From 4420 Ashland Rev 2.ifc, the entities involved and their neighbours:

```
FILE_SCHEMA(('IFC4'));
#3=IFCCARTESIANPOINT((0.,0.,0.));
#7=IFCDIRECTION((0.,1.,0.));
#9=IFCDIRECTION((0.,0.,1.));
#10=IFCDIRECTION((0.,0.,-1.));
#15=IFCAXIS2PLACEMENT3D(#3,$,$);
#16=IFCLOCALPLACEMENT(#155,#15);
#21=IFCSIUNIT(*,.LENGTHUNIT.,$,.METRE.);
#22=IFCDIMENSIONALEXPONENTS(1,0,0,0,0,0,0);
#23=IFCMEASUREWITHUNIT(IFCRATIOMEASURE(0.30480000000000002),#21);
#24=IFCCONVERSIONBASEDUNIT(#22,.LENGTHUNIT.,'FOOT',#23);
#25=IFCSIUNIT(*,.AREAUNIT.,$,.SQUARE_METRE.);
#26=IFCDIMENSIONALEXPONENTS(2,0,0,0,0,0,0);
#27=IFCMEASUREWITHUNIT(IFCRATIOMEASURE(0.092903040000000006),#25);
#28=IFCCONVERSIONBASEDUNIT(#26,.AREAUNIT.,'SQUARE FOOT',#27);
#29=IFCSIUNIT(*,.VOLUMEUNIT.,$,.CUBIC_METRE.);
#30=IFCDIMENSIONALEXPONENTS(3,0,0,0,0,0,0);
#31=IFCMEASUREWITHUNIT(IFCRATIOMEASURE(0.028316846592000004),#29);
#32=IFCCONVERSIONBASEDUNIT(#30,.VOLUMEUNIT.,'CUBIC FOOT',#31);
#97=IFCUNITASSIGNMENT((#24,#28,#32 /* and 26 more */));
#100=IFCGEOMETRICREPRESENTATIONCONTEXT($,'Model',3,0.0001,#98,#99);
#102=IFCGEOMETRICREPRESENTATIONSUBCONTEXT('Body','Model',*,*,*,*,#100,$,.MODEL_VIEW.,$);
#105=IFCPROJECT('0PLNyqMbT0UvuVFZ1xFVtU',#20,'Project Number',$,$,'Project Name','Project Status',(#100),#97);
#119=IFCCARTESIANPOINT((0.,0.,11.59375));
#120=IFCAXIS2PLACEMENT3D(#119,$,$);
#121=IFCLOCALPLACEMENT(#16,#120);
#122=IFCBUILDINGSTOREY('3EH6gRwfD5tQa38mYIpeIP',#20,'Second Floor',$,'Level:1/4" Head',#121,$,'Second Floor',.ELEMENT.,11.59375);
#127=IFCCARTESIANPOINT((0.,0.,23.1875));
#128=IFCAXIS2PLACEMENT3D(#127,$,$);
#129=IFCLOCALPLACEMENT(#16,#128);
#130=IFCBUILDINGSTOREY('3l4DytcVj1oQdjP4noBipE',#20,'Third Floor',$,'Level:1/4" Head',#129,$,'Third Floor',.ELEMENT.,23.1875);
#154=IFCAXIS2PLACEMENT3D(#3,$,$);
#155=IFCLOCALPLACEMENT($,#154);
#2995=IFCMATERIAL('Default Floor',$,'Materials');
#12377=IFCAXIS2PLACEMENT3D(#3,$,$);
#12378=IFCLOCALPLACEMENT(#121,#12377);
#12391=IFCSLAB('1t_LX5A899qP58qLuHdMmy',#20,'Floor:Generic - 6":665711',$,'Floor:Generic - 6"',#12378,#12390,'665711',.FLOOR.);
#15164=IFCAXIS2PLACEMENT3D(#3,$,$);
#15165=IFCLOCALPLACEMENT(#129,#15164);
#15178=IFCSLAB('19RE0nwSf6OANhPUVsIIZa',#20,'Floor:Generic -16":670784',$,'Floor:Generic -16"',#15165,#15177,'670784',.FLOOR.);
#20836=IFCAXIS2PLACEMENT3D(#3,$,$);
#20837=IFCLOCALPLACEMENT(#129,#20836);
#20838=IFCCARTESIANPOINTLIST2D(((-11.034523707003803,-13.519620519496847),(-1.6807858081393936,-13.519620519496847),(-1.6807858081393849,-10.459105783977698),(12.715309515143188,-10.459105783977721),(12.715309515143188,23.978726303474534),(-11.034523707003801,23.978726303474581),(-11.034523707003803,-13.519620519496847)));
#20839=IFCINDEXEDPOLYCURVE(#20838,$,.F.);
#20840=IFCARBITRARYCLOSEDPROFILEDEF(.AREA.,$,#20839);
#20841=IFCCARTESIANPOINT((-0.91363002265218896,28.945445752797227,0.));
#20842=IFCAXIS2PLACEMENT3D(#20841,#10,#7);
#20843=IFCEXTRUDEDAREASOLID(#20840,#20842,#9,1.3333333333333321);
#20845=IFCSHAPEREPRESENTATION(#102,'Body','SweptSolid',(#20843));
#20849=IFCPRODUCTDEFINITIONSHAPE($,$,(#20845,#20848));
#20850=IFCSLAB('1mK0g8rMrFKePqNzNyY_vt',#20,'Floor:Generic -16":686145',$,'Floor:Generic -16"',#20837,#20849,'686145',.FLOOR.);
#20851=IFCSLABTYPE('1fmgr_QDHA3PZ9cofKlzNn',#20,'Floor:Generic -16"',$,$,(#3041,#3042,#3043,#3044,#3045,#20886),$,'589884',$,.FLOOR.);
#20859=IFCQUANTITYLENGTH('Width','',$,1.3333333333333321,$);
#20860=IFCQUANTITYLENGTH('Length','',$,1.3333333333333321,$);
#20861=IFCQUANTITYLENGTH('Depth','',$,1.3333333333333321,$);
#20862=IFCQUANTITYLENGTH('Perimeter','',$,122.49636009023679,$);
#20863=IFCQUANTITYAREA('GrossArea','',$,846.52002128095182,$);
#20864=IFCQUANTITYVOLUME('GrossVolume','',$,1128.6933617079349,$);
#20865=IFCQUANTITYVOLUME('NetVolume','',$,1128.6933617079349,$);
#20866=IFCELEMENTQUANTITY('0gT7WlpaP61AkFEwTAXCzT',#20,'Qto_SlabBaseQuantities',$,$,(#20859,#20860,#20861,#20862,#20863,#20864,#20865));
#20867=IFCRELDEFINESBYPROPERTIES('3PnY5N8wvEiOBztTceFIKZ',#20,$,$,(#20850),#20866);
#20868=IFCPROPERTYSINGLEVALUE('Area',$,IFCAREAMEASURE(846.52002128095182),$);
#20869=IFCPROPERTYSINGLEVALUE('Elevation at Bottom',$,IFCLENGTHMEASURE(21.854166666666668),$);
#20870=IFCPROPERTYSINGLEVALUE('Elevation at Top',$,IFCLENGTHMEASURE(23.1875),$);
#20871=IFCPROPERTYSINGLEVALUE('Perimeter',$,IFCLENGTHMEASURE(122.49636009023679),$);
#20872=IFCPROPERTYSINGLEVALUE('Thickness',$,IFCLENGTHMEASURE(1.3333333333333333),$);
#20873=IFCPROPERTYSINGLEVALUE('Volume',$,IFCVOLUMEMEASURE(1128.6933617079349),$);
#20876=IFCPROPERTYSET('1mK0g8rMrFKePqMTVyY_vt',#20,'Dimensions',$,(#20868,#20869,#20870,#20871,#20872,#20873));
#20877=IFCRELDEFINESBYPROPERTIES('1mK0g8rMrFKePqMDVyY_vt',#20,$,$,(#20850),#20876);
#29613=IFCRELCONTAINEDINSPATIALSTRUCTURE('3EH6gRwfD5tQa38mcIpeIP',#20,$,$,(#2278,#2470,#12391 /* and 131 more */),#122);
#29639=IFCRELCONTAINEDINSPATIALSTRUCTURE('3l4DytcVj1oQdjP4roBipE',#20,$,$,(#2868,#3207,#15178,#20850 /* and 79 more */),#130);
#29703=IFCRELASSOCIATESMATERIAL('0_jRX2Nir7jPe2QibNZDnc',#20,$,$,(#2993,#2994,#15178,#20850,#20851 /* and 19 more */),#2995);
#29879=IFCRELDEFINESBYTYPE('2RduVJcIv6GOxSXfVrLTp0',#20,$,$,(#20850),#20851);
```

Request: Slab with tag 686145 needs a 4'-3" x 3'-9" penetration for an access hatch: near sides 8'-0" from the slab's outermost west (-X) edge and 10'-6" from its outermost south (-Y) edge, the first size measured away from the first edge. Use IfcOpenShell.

```python
import numpy as np
import ifcopenshell
import ifcopenshell.api.feature
import ifcopenshell.api.geometry
import ifcopenshell.api.pset
import ifcopenshell.api.root
import ifcopenshell.geom
import ifcopenshell.util.element
import ifcopenshell.util.placement
import ifcopenshell.util.representation
import ifcopenshell.util.shape
import ifcopenshell.util.unit

model = ifcopenshell.open("4420 Ashland Rev 2.ifc")
unit_scale = ifcopenshell.util.unit.calculate_unit_scale(model)
area_scale = ifcopenshell.util.unit.calculate_unit_scale(model, "AREAUNIT")
volume_scale = ifcopenshell.util.unit.calculate_unit_scale(model, "VOLUMEUNIT")
settings = ifcopenshell.geom.settings()


def volume(element):
    """Net volume in cubic metres, openings subtracted."""
    shape = ifcopenshell.geom.create_shape(settings, element)
    return ifcopenshell.util.shape.get_volume(shape.geometry)


slab = model.by_guid("1mK0g8rMrFKePqNzNyY_vt")
before = volume(slab)

# Extent in the slab's own axes, in metres. The edges named are its -X and -Y sides.
slab_shape = ifcopenshell.geom.create_shape(settings, slab)
vertices = ifcopenshell.util.shape.get_vertices(slab_shape.geometry)
x_min, y_min, bottom = vertices.min(axis=0)
top = vertices[:, 2].max()

opening = ifcopenshell.api.root.create_entity(model, ifc_class="IfcOpeningElement", name="Access hatch opening", predefined_type="OPENING")
context = ifcopenshell.util.representation.get_context(model, "Model", "Body", "MODEL_VIEW")
width, depth = 1.2954, 1.143
outline = [(0.0, 0.0), (width, 0.0), (width, depth), (0.0, depth), (0.0, 0.0)]
# Overshoot both faces by 50 mm so the cut is clean.
shape = ifcopenshell.api.geometry.add_slab_representation(
    model, context=context, depth=top - bottom + 0.1, polyline=outline
)
ifcopenshell.api.geometry.assign_representation(model, product=opening, representation=shape)

matrix = ifcopenshell.util.placement.get_local_placement(slab.ObjectPlacement)
matrix[:, 3] = matrix @ np.append(np.array([x_min + 2.4384, y_min + 3.2004, bottom - 0.05]) / unit_scale, 1.0)
ifcopenshell.api.geometry.edit_object_placement(model, product=opening, matrix=matrix, is_si=False)
ifcopenshell.api.feature.add_feature(model, feature=opening, element=slab)

after = volume(slab)

# Update the slab's stored quantities.
qto = model.by_id(ifcopenshell.util.element.get_pset(slab, "Qto_SlabBaseQuantities", should_inherit=False)["id"])
ifcopenshell.api.pset.edit_qto(model, qto=qto, properties={"NetVolume": after / volume_scale})
pset = model.by_id(ifcopenshell.util.element.get_pset(slab, "Dimensions", should_inherit=False)["id"])
ifcopenshell.api.pset.edit_pset(model, pset=pset, properties={
    "Area": model.create_entity("IfcAreaMeasure", after / (top - bottom) / area_scale),
    "Volume": model.create_entity("IfcVolumeMeasure", after / volume_scale),
})

print(f"slab volume {before:.3f} -> {after:.3f} m3")

model.write("4420 Ashland Rev 2_v2.ifc")
```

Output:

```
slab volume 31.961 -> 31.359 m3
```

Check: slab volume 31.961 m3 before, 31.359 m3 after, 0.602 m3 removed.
